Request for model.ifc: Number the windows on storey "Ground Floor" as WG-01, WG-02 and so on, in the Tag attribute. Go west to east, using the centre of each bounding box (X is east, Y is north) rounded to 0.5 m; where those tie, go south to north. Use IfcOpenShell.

First a look at what the model holds.

```python
import ifcopenshell
import ifcopenshell.util.element
import ifcopenshell.util.placement

model = ifcopenshell.open("model.ifc")
print(model.schema)
storey = next(s for s in model.by_type("IfcBuildingStorey") if s.Name == "Ground Floor")
windows = [e for e in ifcopenshell.util.element.get_decomposition(storey) if e.is_a("IfcWindow")]
for e in sorted(windows, key=lambda e: e.id()):
    origin = ifcopenshell.util.placement.get_local_placement(e.ObjectPlacement)[:3, 3]
    print(e.id(), e.Tag, e.Name, origin.round(2) + 0.0, sep=" | ")
```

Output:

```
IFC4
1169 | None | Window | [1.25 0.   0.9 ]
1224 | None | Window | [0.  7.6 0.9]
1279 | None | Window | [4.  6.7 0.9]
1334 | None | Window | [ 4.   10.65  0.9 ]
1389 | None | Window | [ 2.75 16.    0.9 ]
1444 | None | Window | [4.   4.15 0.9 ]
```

```python
import ifcopenshell
import ifcopenshell.geom
import ifcopenshell.util.element
import ifcopenshell.util.shape

model = ifcopenshell.open("model.ifc")
settings = ifcopenshell.geom.settings()
settings.set("use-world-coords", True)


def centre(element):
    shape = ifcopenshell.geom.create_shape(settings, element)
    return ifcopenshell.util.shape.get_bbox_centroid(shape.geometry)


storey = next(s for s in model.by_type("IfcBuildingStorey") if s.Name == "Ground Floor")
windows = [e for e in ifcopenshell.util.element.get_decomposition(storey) if e.is_a("IfcWindow")]

# Insertion points can sit at a corner or the storey origin, so sort by the geometry (in metres).
centres = {e: centre(e) for e in windows}
windows.sort(key=lambda e: (round(centres[e][0] / 0.5), centres[e][1]))

for i, e in enumerate(windows, start=1):
    number = f"WG-{i:02d}"
    e.Tag = number
    print(e.id(), number)

model.write("model-out.ifc")
```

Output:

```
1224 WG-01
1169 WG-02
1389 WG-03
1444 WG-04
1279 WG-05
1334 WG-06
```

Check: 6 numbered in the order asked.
